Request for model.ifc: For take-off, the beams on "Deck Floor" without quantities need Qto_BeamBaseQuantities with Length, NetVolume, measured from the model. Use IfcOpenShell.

First a look at what the model holds.

```python
import ifcopenshell
import ifcopenshell.util.element
import ifcopenshell.util.unit

model = ifcopenshell.open("model.ifc")
print(model.schema)
for unit_type in ("LENGTHUNIT", "AREAUNIT", "VOLUMEUNIT"):
    print(unit_type, ifcopenshell.util.unit.calculate_unit_scale(model, unit_type))
storey = next(s for s in model.by_type("IfcBuildingStorey") if s.Name == "Deck Floor")
beams = [e for e in ifcopenshell.util.element.get_decomposition(storey) if e.is_a("IfcBeam")]
for e in sorted(beams, key=lambda e: e.id()):
    print(e.id(), e.is_a(), e.Name, list(ifcopenshell.util.element.get_psets(e, qtos_only=True)), sep=" | ")
```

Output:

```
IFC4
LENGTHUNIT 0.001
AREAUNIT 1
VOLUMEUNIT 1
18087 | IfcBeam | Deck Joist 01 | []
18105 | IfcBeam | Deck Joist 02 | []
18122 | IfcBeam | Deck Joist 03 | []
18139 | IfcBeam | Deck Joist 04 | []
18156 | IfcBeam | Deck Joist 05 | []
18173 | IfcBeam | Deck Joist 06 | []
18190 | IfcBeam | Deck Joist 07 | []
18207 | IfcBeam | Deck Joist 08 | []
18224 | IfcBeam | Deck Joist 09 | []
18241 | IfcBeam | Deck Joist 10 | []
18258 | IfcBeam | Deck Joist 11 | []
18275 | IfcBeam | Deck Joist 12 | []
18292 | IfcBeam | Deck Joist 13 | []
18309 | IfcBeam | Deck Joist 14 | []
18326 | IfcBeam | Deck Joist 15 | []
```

```python
import ifcopenshell
import ifcopenshell.api.pset
import ifcopenshell.geom
import ifcopenshell.util.element
import ifcopenshell.util.shape
import ifcopenshell.util.unit

model = ifcopenshell.open("model.ifc")
unit_scale = ifcopenshell.util.unit.calculate_unit_scale(model)
volume_scale = ifcopenshell.util.unit.calculate_unit_scale(model, "VOLUMEUNIT")
settings = ifcopenshell.geom.settings()

storey = next(s for s in model.by_type("IfcBuildingStorey") if s.Name == "Deck Floor")
beams = [e for e in ifcopenshell.util.element.get_decomposition(storey) if e.is_a("IfcBeam")]

for e in sorted(beams, key=lambda e: e.id()):
    if ifcopenshell.util.element.get_psets(e, qtos_only=True, should_inherit=False):
        continue
    # Geometry comes back in metres, in the element's own axes.
    shape = ifcopenshell.geom.create_shape(settings, e)
    values = {
        "Length": ifcopenshell.util.shape.get_max_xyz(shape.geometry) / unit_scale,
        "NetVolume": ifcopenshell.util.shape.get_volume(shape.geometry) / volume_scale,
    }
    qto = ifcopenshell.api.pset.add_qto(model, product=e, name="Qto_BeamBaseQuantities")
    ifcopenshell.api.pset.edit_qto(model, qto=qto, properties=values)
    print(e.id(), {k: round(v, 3) for k, v in values.items()})

model.write("model_updated.ifc")
```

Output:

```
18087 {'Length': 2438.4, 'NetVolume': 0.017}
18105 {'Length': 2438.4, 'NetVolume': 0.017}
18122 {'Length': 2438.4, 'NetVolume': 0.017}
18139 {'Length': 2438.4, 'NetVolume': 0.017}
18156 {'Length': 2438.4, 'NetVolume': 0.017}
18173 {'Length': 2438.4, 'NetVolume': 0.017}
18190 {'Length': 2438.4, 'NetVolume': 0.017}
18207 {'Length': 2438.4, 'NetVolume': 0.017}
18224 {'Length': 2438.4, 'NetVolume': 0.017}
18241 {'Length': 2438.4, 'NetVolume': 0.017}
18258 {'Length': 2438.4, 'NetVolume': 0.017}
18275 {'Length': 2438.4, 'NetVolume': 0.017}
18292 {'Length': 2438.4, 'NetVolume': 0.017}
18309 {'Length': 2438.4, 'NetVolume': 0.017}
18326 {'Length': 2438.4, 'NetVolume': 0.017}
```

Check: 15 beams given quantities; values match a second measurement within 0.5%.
